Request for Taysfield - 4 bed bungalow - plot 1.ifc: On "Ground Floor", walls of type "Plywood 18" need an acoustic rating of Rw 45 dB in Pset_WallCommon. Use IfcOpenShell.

First a look at what the model holds.

```python
import ifcopenshell
import ifcopenshell.util.element

model = ifcopenshell.open("Taysfield - 4 bed bungalow - plot 1.ifc")
print(model.schema)
storey = next(s for s in model.by_type("IfcBuildingStorey") if s.Name == "Ground Floor")
walls = [e for e in ifcopenshell.util.element.get_decomposition(storey) if e.is_a("IfcWall")]
seen = {}
for e in walls:
    element_type = ifcopenshell.util.element.get_type(e)
    key = (element_type.Name if element_type != e and element_type else None, ifcopenshell.util.element.get_pset(e, "Pset_WallCommon", "AcousticRating"))
    seen[key] = seen.get(key, 0) + 1
for (name, value), count in sorted(seen.items(), key=str):
    print(count, "x", name, "|", value)
```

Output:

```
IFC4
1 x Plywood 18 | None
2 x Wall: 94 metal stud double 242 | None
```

```python
import ifcopenshell
import ifcopenshell.api.pset
import ifcopenshell.util.element

model = ifcopenshell.open("Taysfield - 4 bed bungalow - plot 1.ifc")

storey = next(s for s in model.by_type("IfcBuildingStorey") if s.Name == "Ground Floor")
walls = [e for e in ifcopenshell.util.element.get_decomposition(storey) if e.is_a("IfcWall")]

count = 0
for e in walls:
    element_type = ifcopenshell.util.element.get_type(e)
    if element_type in (None, e) or element_type.Name != "Plywood 18":
        continue
    # add_pset returns the element's existing set when there is one.
    pset = ifcopenshell.api.pset.add_pset(model, product=e, name="Pset_WallCommon")
    ifcopenshell.api.pset.edit_pset(model, pset=pset, properties={"AcousticRating": "Rw 45 dB"})
    count += 1

print(count, "walls updated")

model.write("Taysfield - 4 bed bungalow - plot 1-out.ifc")
```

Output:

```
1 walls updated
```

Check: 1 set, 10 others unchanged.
